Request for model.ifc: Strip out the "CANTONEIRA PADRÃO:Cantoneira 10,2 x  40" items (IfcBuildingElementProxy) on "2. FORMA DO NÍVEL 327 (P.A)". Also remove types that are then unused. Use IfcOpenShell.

First a look at what the model holds.

```python
import ifcopenshell
import ifcopenshell.util.element

model = ifcopenshell.open("model.ifc")
print(model.schema)
storey = next(s for s in model.by_type("IfcBuildingStorey") if s.Name == "2. FORMA DO NÍVEL 327 (P.A)")
proxies = [e for e in ifcopenshell.util.element.get_decomposition(storey) if e.is_a("IfcBuildingElementProxy")]
seen = {}
for e in proxies:
    element_type = ifcopenshell.util.element.get_type(e)
    name = element_type.Name if element_type not in (None, e) else None
    seen[name] = seen.get(name, 0) + 1
for name, count in sorted(seen.items(), key=str):
    print(count, "x", name)
```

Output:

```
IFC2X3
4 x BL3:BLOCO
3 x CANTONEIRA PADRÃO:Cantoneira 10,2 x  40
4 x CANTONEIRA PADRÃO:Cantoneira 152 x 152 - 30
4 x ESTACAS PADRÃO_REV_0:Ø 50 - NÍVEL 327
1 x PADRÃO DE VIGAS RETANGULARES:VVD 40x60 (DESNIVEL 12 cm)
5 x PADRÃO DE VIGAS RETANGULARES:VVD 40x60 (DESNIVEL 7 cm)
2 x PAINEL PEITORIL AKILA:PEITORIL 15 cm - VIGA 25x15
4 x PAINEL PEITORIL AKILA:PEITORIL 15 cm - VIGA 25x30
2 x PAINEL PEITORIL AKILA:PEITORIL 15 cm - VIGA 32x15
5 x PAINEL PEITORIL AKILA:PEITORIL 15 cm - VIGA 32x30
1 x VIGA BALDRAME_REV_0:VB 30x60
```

```python
import ifcopenshell
import ifcopenshell.api.root
import ifcopenshell.util.element

model = ifcopenshell.open("model.ifc")

storey = next(s for s in model.by_type("IfcBuildingStorey") if s.Name == "2. FORMA DO NÍVEL 327 (P.A)")
proxies = [e for e in ifcopenshell.util.element.get_decomposition(storey) if e.is_a("IfcBuildingElementProxy")]
targets = [e for e in proxies if (t := ifcopenshell.util.element.get_type(e)) not in (None, e) and t.Name == "CANTONEIRA PADRÃO:Cantoneira 10,2 x  40"]
types = {ifcopenshell.util.element.get_type(e) for e in targets} - {None, *targets}

for e in targets:
    ifcopenshell.api.root.remove_product(model, product=e)
print(len(targets), "removed")

unused = [t for t in types if not ifcopenshell.util.element.get_types(t)]
for t in unused:
    ifcopenshell.api.root.remove_product(model, product=t)
print(len(unused), "unused types removed")

model.write("model-out.ifc")
```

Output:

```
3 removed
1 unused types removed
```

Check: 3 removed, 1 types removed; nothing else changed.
